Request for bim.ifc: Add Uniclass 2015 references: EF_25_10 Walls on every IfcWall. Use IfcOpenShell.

First a look at what the model holds.

```python
import ifcopenshell

model = ifcopenshell.open("bim.ifc")
print(model.schema)
print("classifications:", [c.Name for c in model.by_type("IfcClassification")])
for ifc_class in ("IfcDoor", "IfcRoof", "IfcStair", "IfcWall", "IfcWindow"):
    print(ifc_class, len(model.by_type(ifc_class)))
```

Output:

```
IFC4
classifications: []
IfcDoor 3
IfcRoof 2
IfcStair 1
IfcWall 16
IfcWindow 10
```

```python
import ifcopenshell
import ifcopenshell.api.classification

model = ifcopenshell.open("bim.ifc")

system = ifcopenshell.api.classification.add_classification(model, classification="Uniclass 2015")

codes = {
    "IfcWall": ("EF_25_10", "Walls"),
}
for ifc_class, (code, name) in codes.items():
    products = model.by_type(ifc_class)
    ifcopenshell.api.classification.add_reference(
        model, products=products, classification=system, identification=code, name=name
    )
    print(code, len(products))

model.write("bim_rev.ifc")
```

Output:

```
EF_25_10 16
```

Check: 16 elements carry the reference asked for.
